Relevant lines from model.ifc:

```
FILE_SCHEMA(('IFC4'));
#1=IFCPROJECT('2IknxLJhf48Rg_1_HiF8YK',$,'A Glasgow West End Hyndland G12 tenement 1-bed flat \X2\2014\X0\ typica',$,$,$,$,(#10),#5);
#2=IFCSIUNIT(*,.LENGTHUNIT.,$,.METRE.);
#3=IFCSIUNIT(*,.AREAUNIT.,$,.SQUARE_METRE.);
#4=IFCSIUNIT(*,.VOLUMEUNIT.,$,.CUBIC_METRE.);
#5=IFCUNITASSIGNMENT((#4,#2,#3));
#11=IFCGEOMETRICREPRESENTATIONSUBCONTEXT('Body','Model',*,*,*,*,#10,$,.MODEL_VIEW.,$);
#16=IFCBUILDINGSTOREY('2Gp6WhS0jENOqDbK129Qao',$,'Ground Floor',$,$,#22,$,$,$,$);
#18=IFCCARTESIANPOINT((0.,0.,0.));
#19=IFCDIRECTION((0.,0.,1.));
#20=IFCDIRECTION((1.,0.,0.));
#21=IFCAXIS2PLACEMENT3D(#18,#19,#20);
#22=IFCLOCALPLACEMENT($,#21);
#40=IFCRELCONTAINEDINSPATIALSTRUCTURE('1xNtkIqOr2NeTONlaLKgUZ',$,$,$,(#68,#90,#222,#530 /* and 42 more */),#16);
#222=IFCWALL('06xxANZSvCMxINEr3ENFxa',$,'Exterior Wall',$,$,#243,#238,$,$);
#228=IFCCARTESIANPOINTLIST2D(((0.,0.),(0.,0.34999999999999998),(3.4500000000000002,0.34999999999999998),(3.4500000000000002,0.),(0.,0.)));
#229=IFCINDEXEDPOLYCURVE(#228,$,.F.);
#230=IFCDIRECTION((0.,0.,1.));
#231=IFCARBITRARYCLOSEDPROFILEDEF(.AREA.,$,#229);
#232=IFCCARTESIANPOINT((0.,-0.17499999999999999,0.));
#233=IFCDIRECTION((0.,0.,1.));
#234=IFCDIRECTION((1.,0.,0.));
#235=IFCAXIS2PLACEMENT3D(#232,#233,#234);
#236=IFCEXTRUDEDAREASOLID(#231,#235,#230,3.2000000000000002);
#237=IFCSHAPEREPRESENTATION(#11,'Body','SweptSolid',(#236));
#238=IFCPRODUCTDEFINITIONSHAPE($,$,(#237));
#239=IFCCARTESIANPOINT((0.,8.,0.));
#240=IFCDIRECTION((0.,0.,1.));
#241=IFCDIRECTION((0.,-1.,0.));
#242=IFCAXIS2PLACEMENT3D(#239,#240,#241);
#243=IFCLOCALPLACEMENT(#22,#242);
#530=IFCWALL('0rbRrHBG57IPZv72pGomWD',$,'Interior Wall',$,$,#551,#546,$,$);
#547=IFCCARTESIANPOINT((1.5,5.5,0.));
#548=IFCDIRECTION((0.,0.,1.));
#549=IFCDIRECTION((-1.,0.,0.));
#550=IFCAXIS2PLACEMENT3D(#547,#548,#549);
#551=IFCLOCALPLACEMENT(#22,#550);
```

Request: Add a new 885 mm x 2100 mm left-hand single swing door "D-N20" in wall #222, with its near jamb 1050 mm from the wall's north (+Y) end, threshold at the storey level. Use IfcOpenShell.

```python
import numpy as np
import ifcopenshell
import ifcopenshell.api.feature
import ifcopenshell.api.geometry
import ifcopenshell.api.root
import ifcopenshell.api.spatial
import ifcopenshell.geom
import ifcopenshell.util.element
import ifcopenshell.util.placement
import ifcopenshell.util.representation
import ifcopenshell.util.shape
import ifcopenshell.util.unit

model = ifcopenshell.open("model.ifc")
unit_scale = ifcopenshell.util.unit.calculate_unit_scale(model)
settings = ifcopenshell.geom.settings()


def volume(element):
    """Net volume in cubic metres, openings subtracted."""
    shape = ifcopenshell.geom.create_shape(settings, element)
    return ifcopenshell.util.shape.get_volume(shape.geometry)


wall = model.by_id(222)
storey = ifcopenshell.util.element.get_container(wall, ifc_class="IfcBuildingStorey")
context = ifcopenshell.util.representation.get_context(model, "Model", "Body", "MODEL_VIEW")
before = volume(wall)

width, height, from_end, sill = 0.885, 2.1, 1.05, 0.0  # metres

# The wall runs along its own X axis, and the end named is its -X end.
wall_shape = ifcopenshell.geom.create_shape(settings, wall)
x, y, z = ifcopenshell.util.shape.get_vertices(wall_shape.geometry).T
start = x.min() + from_end
face, thickness = float(y.min()), float(y.max() - y.min())
wall_matrix = ifcopenshell.util.placement.get_local_placement(wall.ObjectPlacement)
level = ifcopenshell.util.placement.get_local_placement(storey.ObjectPlacement)[2, 3]


def in_wall(x, y):
    """Placement at x, y metres in the wall's axes, at sill height."""
    matrix = wall_matrix.copy()
    matrix[:, 3] = wall_matrix @ np.array([x / unit_scale, y / unit_scale, 0.0, 1.0])
    matrix[2, 3] = level + sill / unit_scale
    return matrix


# Opening: a box that overshoots both wall faces by 50 mm.
opening = ifcopenshell.api.root.create_entity(model, ifc_class="IfcOpeningElement", predefined_type="OPENING")
box = ifcopenshell.api.geometry.add_wall_representation(
    model, context=context, length=width, height=height, thickness=thickness + 0.1
)
ifcopenshell.api.geometry.assign_representation(model, product=opening, representation=box)
ifcopenshell.api.geometry.edit_object_placement(model, product=opening, matrix=in_wall(start, face - 0.05), is_si=False)
ifcopenshell.api.feature.add_feature(model, feature=opening, element=wall)

door = ifcopenshell.api.root.create_entity(model, ifc_class="IfcDoor", name="D-N20", predefined_type="DOOR")
door.OverallWidth, door.OverallHeight = width / unit_scale, height / unit_scale
door.OperationType = "SINGLE_SWING_LEFT"
body = ifcopenshell.api.geometry.add_door_representation(
    model,
    context=context,
    overall_width=door.OverallWidth,
    overall_height=door.OverallHeight,
    operation_type="SINGLE_SWING_LEFT",
    lining_properties={"LiningDepth": thickness / unit_scale, "ThresholdDepth": thickness / unit_scale},
)
ifcopenshell.api.geometry.assign_representation(model, product=door, representation=body)
ifcopenshell.api.spatial.assign_container(model, products=[door], relating_structure=storey)
ifcopenshell.api.feature.add_filling(model, opening=opening, element=door)

# The lining spans the wall, so the door starts at the wall face.
ifcopenshell.api.geometry.edit_object_placement(model, product=door, matrix=in_wall(start, face), is_si=False)

after = volume(wall)

print(f"wall volume {before:.3f} -> {after:.3f} m3")

model.write("model_rev.ifc")
```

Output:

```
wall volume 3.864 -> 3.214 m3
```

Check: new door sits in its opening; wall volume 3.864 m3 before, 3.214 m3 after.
